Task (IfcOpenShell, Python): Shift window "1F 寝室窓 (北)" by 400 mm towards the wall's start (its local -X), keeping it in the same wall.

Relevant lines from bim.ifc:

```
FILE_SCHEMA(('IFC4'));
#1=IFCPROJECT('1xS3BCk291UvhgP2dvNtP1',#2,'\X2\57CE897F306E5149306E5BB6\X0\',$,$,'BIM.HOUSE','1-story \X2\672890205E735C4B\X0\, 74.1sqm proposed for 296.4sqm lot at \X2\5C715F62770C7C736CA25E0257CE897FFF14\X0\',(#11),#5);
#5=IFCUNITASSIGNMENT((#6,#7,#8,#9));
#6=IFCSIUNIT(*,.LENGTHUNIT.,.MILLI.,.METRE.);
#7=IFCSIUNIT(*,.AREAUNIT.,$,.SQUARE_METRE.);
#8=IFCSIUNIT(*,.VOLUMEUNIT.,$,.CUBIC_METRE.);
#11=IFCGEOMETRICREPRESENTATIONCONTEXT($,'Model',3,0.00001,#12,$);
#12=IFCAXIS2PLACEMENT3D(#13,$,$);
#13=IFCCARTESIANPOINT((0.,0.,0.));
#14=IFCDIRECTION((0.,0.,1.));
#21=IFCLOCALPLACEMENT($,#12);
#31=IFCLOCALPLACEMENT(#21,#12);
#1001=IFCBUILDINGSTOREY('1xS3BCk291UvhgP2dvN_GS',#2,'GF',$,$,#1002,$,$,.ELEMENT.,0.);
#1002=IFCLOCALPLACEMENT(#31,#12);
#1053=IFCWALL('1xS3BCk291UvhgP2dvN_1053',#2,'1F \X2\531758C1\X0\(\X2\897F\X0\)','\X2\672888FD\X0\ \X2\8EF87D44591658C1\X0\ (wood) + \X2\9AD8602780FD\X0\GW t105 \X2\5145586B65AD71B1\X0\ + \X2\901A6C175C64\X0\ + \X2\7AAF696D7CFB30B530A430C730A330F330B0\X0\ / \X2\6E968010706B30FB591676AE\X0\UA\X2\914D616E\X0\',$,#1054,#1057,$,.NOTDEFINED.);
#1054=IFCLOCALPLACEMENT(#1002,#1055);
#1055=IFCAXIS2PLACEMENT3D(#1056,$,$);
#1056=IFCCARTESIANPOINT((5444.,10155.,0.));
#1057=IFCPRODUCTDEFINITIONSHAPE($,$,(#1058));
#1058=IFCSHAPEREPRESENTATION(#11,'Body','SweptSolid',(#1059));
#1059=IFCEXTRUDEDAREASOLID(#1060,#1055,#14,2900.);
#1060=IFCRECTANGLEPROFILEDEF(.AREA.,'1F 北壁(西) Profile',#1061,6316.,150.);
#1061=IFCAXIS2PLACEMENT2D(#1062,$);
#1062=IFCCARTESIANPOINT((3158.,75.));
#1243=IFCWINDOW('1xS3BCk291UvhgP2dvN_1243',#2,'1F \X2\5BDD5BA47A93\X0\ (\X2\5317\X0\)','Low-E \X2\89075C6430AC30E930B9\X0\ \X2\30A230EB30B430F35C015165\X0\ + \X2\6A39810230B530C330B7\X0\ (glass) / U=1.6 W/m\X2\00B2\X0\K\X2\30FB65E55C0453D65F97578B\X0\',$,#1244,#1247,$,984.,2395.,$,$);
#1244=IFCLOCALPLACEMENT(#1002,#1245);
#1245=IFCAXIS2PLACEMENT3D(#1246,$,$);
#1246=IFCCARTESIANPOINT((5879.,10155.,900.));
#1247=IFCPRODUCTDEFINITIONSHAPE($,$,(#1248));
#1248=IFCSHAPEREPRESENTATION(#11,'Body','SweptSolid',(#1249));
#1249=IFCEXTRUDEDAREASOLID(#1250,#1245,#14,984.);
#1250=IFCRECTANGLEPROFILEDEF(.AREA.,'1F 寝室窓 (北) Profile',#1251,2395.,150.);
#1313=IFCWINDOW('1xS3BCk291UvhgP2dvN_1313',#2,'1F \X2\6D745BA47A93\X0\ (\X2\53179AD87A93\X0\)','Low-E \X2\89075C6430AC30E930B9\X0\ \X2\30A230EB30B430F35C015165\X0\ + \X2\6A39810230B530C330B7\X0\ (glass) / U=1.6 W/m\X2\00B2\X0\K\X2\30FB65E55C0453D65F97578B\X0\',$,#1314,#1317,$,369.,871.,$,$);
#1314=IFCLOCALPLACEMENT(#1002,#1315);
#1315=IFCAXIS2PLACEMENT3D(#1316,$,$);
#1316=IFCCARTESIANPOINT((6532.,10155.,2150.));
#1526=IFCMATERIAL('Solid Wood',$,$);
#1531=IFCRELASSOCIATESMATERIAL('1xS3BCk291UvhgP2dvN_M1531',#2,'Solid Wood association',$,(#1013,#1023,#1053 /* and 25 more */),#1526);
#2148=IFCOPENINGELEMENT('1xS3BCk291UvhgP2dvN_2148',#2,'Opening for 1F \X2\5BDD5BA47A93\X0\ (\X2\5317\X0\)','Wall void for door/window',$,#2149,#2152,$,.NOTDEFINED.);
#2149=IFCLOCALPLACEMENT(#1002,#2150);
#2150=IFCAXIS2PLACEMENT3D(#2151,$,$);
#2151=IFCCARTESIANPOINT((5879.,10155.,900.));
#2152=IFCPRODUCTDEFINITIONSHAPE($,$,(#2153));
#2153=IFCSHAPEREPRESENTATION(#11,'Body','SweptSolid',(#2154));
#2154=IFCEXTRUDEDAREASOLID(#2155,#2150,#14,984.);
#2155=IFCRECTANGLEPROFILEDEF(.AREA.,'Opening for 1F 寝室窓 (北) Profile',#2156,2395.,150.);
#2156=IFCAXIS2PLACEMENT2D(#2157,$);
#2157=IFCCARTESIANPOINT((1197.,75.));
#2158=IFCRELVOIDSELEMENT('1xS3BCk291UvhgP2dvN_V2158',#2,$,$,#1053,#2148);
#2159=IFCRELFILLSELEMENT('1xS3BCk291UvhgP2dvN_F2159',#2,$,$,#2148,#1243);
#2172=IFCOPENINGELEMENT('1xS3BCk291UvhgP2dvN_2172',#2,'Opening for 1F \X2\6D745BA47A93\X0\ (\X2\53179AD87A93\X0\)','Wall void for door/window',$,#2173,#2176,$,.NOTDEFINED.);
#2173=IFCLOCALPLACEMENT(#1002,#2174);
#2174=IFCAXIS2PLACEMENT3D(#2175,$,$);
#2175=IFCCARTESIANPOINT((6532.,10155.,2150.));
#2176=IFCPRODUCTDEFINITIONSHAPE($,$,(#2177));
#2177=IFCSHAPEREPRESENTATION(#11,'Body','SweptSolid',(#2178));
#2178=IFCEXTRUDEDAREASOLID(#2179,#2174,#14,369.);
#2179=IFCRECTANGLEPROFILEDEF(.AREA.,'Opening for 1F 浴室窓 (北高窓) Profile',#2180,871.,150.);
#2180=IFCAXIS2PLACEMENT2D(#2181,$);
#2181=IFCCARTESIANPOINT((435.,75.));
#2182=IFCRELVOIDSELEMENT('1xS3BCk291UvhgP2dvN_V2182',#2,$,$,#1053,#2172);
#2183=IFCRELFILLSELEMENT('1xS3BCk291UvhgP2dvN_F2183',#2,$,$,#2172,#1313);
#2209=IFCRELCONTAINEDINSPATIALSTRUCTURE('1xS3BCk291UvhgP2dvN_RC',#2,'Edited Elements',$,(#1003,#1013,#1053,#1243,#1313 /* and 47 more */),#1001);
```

```python
import ifcopenshell
import ifcopenshell.api.geometry
import ifcopenshell.util.placement

model = ifcopenshell.open("bim.ifc")

window = model.by_guid("1xS3BCk291UvhgP2dvN_1243")
opening = window.FillsVoids[0].RelatingOpeningElement
wall = opening.VoidsElements[0].RelatingBuildingElement

wall_matrix = ifcopenshell.util.placement.get_local_placement(wall.ObjectPlacement)
shift = wall_matrix[:3, 0] * -400.0
before = ifcopenshell.util.placement.get_local_placement(window.ObjectPlacement)[:3, 3].copy()

# The window is not placed relative to its opening, so move both.
for product in (opening, window):
    matrix = ifcopenshell.util.placement.get_local_placement(product.ObjectPlacement)
    matrix[:3, 3] += shift
    ifcopenshell.api.geometry.edit_object_placement(model, product=product, matrix=matrix, is_si=False)

after = ifcopenshell.util.placement.get_local_placement(window.ObjectPlacement)[:3, 3]
print("window moved by", (after - before).round(3) + 0.0)

model.write("bim_rev.ifc")
```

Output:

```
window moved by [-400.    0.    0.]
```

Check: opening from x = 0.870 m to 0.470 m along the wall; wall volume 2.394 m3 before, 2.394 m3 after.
